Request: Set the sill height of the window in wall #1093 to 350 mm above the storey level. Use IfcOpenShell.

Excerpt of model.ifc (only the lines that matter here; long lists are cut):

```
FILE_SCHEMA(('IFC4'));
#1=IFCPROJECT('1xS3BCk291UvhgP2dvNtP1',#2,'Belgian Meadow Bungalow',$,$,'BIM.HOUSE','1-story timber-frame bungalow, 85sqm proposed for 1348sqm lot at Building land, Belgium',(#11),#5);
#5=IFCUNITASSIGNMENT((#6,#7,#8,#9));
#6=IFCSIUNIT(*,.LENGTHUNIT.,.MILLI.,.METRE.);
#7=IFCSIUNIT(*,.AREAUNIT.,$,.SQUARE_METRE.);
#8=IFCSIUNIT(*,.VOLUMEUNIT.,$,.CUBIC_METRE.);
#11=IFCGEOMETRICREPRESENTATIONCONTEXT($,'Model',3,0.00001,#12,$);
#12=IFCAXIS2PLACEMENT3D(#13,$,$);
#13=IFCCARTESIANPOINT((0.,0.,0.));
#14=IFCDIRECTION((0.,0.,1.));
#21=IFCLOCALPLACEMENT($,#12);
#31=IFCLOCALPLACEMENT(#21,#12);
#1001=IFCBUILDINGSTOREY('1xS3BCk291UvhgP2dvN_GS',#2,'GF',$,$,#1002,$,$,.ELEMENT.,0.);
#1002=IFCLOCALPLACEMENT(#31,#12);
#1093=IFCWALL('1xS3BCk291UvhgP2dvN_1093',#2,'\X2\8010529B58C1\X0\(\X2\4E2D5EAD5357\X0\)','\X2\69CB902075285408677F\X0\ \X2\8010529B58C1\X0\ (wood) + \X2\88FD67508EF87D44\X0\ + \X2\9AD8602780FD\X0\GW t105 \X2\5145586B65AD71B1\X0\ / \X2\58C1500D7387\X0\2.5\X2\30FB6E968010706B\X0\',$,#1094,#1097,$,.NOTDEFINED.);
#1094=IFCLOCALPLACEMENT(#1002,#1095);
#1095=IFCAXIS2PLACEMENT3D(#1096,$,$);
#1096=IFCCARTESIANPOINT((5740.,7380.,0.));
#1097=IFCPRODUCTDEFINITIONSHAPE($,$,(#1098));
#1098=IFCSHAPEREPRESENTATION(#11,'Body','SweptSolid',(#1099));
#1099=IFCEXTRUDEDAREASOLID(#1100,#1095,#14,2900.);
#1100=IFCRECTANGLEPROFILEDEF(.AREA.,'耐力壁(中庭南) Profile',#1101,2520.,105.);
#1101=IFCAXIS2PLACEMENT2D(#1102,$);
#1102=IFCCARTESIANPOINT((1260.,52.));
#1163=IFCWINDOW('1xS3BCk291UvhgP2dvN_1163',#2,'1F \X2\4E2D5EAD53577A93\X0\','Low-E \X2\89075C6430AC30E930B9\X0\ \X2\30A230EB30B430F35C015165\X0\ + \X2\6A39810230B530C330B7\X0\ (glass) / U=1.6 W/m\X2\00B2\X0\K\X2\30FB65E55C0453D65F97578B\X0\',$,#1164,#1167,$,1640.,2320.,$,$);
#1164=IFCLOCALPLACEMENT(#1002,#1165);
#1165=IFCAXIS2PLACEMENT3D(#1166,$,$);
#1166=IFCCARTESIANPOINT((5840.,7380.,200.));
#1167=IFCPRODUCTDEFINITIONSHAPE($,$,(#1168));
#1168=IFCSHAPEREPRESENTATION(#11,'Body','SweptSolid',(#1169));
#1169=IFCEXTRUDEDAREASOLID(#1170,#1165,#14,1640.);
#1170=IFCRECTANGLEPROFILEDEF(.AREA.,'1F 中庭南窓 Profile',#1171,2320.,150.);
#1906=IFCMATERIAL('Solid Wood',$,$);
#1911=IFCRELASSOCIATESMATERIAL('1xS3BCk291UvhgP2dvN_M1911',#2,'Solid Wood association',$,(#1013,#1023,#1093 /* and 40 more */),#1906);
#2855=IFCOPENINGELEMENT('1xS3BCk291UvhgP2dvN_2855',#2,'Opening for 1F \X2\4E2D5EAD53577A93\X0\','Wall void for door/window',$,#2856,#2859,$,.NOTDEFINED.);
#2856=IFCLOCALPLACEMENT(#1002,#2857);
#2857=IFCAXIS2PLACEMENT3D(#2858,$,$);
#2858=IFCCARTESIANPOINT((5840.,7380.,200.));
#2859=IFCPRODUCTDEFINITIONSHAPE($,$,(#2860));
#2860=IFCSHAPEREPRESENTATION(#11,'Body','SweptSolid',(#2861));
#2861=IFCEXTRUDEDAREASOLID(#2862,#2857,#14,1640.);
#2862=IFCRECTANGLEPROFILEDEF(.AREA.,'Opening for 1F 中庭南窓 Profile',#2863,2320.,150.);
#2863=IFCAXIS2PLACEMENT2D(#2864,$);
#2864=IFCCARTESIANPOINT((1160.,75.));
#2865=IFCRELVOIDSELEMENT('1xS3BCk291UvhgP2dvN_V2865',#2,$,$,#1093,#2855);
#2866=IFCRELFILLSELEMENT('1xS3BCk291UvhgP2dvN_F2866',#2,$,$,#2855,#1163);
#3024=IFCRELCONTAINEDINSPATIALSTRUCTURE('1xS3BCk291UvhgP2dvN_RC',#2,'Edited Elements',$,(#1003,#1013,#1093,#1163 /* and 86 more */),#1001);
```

```python
import numpy as np
import ifcopenshell
import ifcopenshell.api.geometry
import ifcopenshell.geom
import ifcopenshell.util.element
import ifcopenshell.util.placement
import ifcopenshell.util.shape
import ifcopenshell.util.unit

model = ifcopenshell.open("model.ifc")
unit_scale = ifcopenshell.util.unit.calculate_unit_scale(model)

window = model.by_id(1163)
opening = window.FillsVoids[0].RelatingOpeningElement
storey = ifcopenshell.util.element.get_container(window, ifc_class="IfcBuildingStorey")
level = ifcopenshell.util.placement.get_local_placement(storey.ObjectPlacement)[2, 3]

# The opening's origin need not be at the sill, so measure its lowest point.
shape = ifcopenshell.geom.create_shape(ifcopenshell.geom.settings(), opening)
bottom = ifcopenshell.util.shape.get_shape_bottom_elevation(shape, shape.geometry) / unit_scale
dz = level + 0.35 / unit_scale - bottom

shift = np.array([0.0, 0.0, dz])
# The window is not placed relative to its opening, so move both.
for product in (opening, window):
    matrix = ifcopenshell.util.placement.get_local_placement(product.ObjectPlacement)
    matrix[:3, 3] += shift
    ifcopenshell.api.geometry.edit_object_placement(model, product=product, matrix=matrix, is_si=False)

print(f"moved by {dz * unit_scale:+.3f} m")

model.write("model_edited.ifc")
```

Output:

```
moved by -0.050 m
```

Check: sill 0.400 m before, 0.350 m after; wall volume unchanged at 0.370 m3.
